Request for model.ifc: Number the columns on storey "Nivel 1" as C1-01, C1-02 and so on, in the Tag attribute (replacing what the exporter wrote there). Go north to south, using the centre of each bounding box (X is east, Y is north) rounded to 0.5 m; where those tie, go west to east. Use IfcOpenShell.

First a look at what the model holds.

```python
import ifcopenshell
import ifcopenshell.util.element
import ifcopenshell.util.placement

model = ifcopenshell.open("model.ifc")
print(model.schema)
storey = next(s for s in model.by_type("IfcBuildingStorey") if s.Name == "Nivel 1")
columns = [e for e in ifcopenshell.util.element.get_decomposition(storey) if e.is_a("IfcColumn")]
for e in sorted(columns, key=lambda e: e.id()):
    origin = ifcopenshell.util.placement.get_local_placement(e.ObjectPlacement)[:3, 3]
    print(e.id(), e.Tag, e.Name, origin.round(2) + 0.0, sep=" | ")
```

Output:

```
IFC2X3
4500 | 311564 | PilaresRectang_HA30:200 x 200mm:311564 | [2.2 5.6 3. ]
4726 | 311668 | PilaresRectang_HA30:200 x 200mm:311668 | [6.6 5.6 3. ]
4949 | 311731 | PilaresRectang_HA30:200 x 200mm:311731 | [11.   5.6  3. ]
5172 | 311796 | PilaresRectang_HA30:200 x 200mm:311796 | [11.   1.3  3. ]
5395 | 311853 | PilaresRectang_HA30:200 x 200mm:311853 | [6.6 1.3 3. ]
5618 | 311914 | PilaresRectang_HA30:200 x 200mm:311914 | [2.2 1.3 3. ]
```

```python
import ifcopenshell
import ifcopenshell.geom
import ifcopenshell.util.element
import ifcopenshell.util.shape

model = ifcopenshell.open("model.ifc")
settings = ifcopenshell.geom.settings()
settings.set("use-world-coords", True)


def centre(element):
    shape = ifcopenshell.geom.create_shape(settings, element)
    return ifcopenshell.util.shape.get_bbox_centroid(shape.geometry)


storey = next(s for s in model.by_type("IfcBuildingStorey") if s.Name == "Nivel 1")
columns = [e for e in ifcopenshell.util.element.get_decomposition(storey) if e.is_a("IfcColumn")]

# Insertion points can sit at a corner or the storey origin, so sort by the geometry (in metres).
centres = {e: centre(e) for e in columns}
columns.sort(key=lambda e: (-round(centres[e][1] / 0.5), centres[e][0]))

for i, e in enumerate(columns, start=1):
    number = f"C1-{i:02d}"
    e.Tag = number
    print(e.id(), number)

model.write("model_rev.ifc")
```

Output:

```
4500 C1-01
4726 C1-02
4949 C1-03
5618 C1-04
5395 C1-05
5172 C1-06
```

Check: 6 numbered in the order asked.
